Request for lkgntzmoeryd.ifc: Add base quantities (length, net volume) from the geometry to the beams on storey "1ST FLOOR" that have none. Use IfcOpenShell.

First a look at what the model holds.

```python
import ifcopenshell
import ifcopenshell.util.element
import ifcopenshell.util.unit

model = ifcopenshell.open("lkgntzmoeryd.ifc")
print(model.schema)
for unit_type in ("LENGTHUNIT", "AREAUNIT", "VOLUMEUNIT"):
    print(unit_type, ifcopenshell.util.unit.calculate_unit_scale(model, unit_type))
storey = next(s for s in model.by_type("IfcBuildingStorey") if s.Name == "1ST FLOOR")
beams = [e for e in ifcopenshell.util.element.get_decomposition(storey) if e.is_a("IfcBeam")]
for e in sorted(beams, key=lambda e: e.id()):
    print(e.id(), e.is_a(), e.Name, list(ifcopenshell.util.element.get_psets(e, qtos_only=True)), sep=" | ")
```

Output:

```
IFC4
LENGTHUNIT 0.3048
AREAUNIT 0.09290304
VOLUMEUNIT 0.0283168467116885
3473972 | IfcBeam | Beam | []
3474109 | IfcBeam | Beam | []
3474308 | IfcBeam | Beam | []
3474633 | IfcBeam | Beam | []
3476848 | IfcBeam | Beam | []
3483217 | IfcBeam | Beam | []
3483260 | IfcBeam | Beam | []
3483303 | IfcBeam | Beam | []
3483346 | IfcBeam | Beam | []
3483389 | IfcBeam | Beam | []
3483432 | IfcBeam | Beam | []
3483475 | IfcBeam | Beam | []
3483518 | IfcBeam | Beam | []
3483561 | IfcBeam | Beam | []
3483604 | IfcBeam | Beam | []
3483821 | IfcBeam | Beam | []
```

```python
import ifcopenshell
import ifcopenshell.api.pset
import ifcopenshell.geom
import ifcopenshell.util.element
import ifcopenshell.util.shape
import ifcopenshell.util.unit

model = ifcopenshell.open("lkgntzmoeryd.ifc")
unit_scale = ifcopenshell.util.unit.calculate_unit_scale(model)
volume_scale = ifcopenshell.util.unit.calculate_unit_scale(model, "VOLUMEUNIT")
settings = ifcopenshell.geom.settings()

storey = next(s for s in model.by_type("IfcBuildingStorey") if s.Name == "1ST FLOOR")
beams = [e for e in ifcopenshell.util.element.get_decomposition(storey) if e.is_a("IfcBeam")]

for e in sorted(beams, key=lambda e: e.id()):
    if ifcopenshell.util.element.get_psets(e, qtos_only=True, should_inherit=False):
        continue
    # Geometry comes back in metres, in the element's own axes.
    shape = ifcopenshell.geom.create_shape(settings, e)
    values = {
        "Length": ifcopenshell.util.shape.get_max_xyz(shape.geometry) / unit_scale,
        "NetVolume": ifcopenshell.util.shape.get_volume(shape.geometry) / volume_scale,
    }
    qto = ifcopenshell.api.pset.add_qto(model, product=e, name="Qto_BeamBaseQuantities")
    ifcopenshell.api.pset.edit_qto(model, qto=qto, properties=values)
    print(e.id(), {k: round(v, 3) for k, v in values.items()})

model.write("lkgntzmoeryd-out.ifc")
```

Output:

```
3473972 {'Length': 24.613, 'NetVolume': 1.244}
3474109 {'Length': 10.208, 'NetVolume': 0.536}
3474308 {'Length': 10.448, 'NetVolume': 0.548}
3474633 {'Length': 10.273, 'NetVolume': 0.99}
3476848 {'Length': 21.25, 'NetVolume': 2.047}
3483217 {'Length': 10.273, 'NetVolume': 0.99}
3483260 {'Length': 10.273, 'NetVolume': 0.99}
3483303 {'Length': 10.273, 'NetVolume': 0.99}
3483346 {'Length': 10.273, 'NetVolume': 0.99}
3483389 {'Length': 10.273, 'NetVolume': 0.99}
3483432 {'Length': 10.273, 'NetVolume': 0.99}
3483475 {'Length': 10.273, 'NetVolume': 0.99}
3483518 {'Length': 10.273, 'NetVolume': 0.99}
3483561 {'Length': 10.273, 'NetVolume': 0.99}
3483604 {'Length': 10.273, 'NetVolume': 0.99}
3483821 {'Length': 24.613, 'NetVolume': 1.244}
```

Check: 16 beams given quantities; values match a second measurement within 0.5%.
